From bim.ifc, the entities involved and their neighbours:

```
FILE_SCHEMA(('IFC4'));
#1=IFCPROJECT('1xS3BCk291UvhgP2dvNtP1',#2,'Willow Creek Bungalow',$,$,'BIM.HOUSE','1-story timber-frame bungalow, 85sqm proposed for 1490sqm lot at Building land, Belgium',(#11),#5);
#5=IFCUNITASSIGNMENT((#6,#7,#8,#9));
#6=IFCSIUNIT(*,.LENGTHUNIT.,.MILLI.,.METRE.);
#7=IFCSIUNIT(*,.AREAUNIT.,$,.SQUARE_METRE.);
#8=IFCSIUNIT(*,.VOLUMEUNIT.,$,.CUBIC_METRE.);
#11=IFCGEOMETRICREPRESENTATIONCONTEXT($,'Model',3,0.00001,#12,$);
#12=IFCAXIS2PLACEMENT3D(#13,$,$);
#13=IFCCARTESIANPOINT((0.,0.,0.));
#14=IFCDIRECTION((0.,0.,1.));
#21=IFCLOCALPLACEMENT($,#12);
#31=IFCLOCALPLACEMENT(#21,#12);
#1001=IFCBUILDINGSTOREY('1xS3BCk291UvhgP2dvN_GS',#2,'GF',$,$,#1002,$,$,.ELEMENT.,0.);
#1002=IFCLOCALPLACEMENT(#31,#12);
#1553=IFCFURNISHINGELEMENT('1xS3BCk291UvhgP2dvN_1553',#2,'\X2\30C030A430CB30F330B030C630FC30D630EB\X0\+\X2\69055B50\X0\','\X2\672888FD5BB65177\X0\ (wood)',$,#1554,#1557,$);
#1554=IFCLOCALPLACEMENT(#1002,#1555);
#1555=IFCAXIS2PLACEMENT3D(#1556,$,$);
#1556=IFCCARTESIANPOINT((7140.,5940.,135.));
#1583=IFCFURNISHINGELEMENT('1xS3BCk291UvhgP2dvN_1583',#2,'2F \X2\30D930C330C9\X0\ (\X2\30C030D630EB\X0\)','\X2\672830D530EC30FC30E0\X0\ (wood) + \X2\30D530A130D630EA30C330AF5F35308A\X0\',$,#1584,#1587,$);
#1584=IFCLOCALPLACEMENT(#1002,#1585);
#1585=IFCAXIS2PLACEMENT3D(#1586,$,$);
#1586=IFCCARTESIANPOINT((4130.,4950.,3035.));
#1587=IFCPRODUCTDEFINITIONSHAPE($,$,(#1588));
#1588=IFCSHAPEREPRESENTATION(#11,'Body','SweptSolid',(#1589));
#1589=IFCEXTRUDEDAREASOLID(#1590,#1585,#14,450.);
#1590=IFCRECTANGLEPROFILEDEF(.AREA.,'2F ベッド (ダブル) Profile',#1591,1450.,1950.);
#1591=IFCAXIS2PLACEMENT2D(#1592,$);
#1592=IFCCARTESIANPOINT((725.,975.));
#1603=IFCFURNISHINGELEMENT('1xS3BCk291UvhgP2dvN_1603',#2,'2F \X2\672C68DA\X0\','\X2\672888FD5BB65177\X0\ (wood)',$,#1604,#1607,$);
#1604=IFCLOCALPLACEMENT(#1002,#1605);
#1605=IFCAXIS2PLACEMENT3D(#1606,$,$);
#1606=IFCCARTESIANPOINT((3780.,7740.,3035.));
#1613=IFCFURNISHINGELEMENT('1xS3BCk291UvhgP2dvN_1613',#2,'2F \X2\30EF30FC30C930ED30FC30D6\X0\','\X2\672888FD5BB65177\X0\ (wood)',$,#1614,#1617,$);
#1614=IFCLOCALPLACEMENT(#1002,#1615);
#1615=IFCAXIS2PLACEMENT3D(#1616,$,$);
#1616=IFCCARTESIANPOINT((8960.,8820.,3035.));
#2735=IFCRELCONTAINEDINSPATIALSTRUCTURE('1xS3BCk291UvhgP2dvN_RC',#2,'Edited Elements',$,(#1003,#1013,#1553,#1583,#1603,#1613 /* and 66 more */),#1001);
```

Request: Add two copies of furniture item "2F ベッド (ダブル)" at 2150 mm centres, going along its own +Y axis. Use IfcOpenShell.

```python
import ifcopenshell
import ifcopenshell.api.geometry
import ifcopenshell.api.root
import ifcopenshell.util.element
import ifcopenshell.util.placement
import ifcopenshell.util.unit

model = ifcopenshell.open("bim.ifc")
unit_scale = ifcopenshell.util.unit.calculate_unit_scale(model)


def reuse_history(source, copy):
    """copy_class also copies each property set's owner history, people and application; keep the originals."""
    for rel in copy.IsDefinedBy:
        if rel.is_a("IfcRelDefinesByProperties") and (history := rel.RelatingPropertyDefinition.OwnerHistory):
            rel.RelatingPropertyDefinition.OwnerHistory = source.OwnerHistory
            ifcopenshell.util.element.remove_deep2(model, history)


source = model.by_guid("1xS3BCk291UvhgP2dvN_1583")
base = ifcopenshell.util.placement.get_local_placement(source.ObjectPlacement)
step = base[:3, 1] * 2.15 / unit_scale

for i in range(1, 3):
    copy = ifcopenshell.api.root.copy_class(model, product=source)
    copy.Representation = ifcopenshell.util.element.copy_deep(
        model, source.Representation, exclude=["IfcGeometricRepresentationContext", "IfcRepresentationMap"]
    )
    reuse_history(source, copy)
    matrix = base.copy()
    matrix[:3, 3] += i * step
    print("added at", matrix[:3, 3].round(3) + 0.0)
    ifcopenshell.api.geometry.edit_object_placement(model, product=copy, matrix=matrix, is_si=False)

model.write("bim_edited.ifc")
```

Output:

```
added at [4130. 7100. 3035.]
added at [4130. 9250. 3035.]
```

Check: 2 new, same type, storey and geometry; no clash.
